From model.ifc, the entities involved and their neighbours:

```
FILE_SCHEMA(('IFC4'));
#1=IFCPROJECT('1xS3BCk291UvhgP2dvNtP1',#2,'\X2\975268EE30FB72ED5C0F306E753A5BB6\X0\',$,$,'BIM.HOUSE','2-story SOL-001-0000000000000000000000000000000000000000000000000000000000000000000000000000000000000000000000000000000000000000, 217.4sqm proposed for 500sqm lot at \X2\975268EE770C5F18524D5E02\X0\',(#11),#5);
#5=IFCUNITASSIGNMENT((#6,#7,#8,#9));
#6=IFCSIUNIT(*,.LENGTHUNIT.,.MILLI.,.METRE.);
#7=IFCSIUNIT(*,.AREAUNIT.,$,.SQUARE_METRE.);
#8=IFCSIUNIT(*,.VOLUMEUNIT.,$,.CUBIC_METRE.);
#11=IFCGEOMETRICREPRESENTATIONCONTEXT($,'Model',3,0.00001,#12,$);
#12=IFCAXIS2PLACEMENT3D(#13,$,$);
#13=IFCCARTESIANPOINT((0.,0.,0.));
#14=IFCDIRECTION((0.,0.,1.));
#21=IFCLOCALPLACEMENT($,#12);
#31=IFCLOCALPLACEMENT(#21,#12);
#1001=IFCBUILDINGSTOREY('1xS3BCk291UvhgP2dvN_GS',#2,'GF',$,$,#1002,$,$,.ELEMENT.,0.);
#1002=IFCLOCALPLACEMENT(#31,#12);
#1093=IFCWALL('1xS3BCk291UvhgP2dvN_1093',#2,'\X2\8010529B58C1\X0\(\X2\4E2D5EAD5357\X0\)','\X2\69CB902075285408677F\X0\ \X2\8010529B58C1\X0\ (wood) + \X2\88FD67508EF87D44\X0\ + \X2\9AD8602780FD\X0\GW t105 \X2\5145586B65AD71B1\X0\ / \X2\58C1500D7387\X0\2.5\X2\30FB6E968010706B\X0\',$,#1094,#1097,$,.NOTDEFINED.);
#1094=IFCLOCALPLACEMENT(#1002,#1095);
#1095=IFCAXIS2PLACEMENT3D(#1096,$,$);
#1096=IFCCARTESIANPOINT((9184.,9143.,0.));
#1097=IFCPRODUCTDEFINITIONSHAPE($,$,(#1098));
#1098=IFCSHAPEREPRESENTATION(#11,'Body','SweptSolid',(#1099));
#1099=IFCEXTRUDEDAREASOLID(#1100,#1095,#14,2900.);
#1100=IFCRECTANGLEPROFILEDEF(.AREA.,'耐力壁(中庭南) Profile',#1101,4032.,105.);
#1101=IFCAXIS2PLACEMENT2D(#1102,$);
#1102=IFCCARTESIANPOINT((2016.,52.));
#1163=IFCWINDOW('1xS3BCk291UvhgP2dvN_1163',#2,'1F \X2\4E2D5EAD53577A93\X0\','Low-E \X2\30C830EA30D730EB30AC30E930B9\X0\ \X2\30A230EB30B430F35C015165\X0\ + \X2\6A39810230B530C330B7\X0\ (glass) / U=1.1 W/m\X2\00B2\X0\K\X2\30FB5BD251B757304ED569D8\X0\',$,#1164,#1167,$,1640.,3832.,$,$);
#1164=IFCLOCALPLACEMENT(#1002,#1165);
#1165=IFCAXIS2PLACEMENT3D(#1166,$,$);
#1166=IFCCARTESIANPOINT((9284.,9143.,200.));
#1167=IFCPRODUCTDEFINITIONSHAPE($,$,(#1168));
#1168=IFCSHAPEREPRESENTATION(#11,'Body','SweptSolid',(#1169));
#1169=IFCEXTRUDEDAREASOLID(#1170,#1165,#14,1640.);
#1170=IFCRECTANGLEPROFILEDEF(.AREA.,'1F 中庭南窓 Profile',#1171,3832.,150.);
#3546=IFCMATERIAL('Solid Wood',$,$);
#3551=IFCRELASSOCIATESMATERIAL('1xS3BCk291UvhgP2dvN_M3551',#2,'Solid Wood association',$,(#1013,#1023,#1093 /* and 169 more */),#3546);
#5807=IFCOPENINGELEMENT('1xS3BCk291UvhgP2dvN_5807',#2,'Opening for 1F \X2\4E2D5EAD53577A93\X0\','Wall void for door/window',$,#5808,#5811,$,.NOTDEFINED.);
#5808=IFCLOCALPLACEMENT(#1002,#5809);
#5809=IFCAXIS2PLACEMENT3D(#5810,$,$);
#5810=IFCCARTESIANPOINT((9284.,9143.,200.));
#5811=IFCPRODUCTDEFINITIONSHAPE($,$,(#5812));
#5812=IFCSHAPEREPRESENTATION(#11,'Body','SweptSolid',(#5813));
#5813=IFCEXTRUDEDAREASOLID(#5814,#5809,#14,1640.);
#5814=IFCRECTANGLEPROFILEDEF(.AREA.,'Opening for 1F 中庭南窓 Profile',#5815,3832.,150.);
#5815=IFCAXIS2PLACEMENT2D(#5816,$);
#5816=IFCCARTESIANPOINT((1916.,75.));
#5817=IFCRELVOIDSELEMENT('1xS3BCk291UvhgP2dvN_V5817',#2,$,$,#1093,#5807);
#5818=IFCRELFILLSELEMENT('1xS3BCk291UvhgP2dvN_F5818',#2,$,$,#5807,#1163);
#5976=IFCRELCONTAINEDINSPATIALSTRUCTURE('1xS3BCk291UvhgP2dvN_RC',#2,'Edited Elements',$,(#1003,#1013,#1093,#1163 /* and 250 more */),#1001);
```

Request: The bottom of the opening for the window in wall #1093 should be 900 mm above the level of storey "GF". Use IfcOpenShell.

```python
import numpy as np
import ifcopenshell
import ifcopenshell.api.geometry
import ifcopenshell.geom
import ifcopenshell.util.element
import ifcopenshell.util.placement
import ifcopenshell.util.shape
import ifcopenshell.util.unit

model = ifcopenshell.open("model.ifc")
unit_scale = ifcopenshell.util.unit.calculate_unit_scale(model)

window = model.by_guid("1xS3BCk291UvhgP2dvN_1163")
opening = window.FillsVoids[0].RelatingOpeningElement
storey = ifcopenshell.util.element.get_container(window, ifc_class="IfcBuildingStorey")
level = ifcopenshell.util.placement.get_local_placement(storey.ObjectPlacement)[2, 3]

# The opening's origin need not be at the sill, so measure its lowest point.
shape = ifcopenshell.geom.create_shape(ifcopenshell.geom.settings(), opening)
bottom = ifcopenshell.util.shape.get_shape_bottom_elevation(shape, shape.geometry) / unit_scale
dz = level + 0.9 / unit_scale - bottom

shift = np.array([0.0, 0.0, dz])
# The window is not placed relative to its opening, so move both.
for product in (opening, window):
    matrix = ifcopenshell.util.placement.get_local_placement(product.ObjectPlacement)
    matrix[:3, 3] += shift
    ifcopenshell.api.geometry.edit_object_placement(model, product=product, matrix=matrix, is_si=False)

print(f"moved by {dz * unit_scale:+.3f} m")

model.write("model-out.ifc")
```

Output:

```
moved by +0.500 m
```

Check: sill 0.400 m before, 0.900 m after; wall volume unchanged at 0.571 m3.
